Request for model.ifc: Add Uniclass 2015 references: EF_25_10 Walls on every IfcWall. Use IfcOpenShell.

First a look at what the model holds.

```python
import ifcopenshell

model = ifcopenshell.open("model.ifc")
print(model.schema)
print("classifications:", [c.Name for c in model.by_type("IfcClassification")])
for ifc_class in ("IfcDoor", "IfcRoof", "IfcStair", "IfcWall", "IfcWindow"):
    print(ifc_class, len(model.by_type(ifc_class)))
```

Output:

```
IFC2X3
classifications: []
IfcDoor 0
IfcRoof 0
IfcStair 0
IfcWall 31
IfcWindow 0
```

```python
import ifcopenshell
import ifcopenshell.api.classification

model = ifcopenshell.open("model.ifc")

# IFC2X3 requires Source and Edition and has no link from the project to the system.
system = model.create_entity("IfcClassification", Source="NBS", Edition="2015", Name="Uniclass 2015")

codes = {
    "IfcWall": ("EF_25_10", "Walls"),
}
for ifc_class, (code, name) in codes.items():
    products = model.by_type(ifc_class)
    ifcopenshell.api.classification.add_reference(
        model, products=products, classification=system, identification=code, name=name
    )
    print(code, len(products))

model.write("model-out.ifc")
```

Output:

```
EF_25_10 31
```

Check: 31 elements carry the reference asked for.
